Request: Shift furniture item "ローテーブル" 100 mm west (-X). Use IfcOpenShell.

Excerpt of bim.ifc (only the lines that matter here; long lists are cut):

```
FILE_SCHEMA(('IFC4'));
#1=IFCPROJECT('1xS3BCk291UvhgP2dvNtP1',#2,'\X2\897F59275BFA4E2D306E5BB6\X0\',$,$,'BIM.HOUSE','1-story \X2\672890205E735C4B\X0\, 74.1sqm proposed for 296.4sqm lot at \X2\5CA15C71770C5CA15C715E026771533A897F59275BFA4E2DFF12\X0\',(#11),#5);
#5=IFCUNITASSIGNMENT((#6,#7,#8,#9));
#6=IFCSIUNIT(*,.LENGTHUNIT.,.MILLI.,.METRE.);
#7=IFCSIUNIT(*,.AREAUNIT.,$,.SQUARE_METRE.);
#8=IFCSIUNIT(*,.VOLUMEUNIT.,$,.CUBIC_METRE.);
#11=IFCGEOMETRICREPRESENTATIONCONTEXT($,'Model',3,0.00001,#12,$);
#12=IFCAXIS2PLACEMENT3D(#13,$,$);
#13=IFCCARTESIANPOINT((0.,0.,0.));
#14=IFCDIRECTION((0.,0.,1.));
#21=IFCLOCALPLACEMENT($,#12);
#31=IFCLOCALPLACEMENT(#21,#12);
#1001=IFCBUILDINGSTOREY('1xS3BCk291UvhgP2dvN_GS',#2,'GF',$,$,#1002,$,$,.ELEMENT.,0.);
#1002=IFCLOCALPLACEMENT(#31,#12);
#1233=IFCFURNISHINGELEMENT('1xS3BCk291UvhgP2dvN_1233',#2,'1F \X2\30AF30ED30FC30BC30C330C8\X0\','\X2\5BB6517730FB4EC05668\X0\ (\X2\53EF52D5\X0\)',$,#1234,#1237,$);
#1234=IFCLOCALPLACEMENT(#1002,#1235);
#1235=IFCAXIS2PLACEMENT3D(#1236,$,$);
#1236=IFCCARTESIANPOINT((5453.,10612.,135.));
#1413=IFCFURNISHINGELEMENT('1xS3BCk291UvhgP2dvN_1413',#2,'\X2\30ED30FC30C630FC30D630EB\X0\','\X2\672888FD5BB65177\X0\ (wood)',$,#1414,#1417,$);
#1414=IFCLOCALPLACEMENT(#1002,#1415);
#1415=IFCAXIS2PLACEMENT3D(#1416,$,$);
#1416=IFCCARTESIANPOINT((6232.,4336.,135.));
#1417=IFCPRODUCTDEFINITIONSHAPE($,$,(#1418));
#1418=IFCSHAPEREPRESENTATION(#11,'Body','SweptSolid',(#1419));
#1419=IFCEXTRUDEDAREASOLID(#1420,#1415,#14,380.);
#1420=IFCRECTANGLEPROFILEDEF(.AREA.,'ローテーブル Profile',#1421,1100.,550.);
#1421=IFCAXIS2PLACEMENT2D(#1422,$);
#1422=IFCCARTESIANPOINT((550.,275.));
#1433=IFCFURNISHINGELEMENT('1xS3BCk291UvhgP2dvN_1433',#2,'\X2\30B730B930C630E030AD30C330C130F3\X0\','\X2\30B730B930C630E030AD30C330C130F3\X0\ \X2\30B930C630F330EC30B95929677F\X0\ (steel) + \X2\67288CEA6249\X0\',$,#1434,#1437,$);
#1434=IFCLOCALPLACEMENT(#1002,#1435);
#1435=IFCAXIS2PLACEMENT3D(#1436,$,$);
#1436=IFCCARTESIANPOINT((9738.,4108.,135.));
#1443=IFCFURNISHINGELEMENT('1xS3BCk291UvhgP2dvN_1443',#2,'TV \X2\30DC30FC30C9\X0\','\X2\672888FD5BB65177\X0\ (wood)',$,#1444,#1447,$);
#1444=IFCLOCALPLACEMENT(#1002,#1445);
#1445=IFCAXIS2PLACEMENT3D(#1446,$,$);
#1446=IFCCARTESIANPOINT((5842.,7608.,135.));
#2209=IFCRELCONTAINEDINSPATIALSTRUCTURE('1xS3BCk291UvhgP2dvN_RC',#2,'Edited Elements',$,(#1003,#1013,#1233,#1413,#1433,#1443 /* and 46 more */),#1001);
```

```python
import ifcopenshell
import ifcopenshell.api.geometry
import ifcopenshell.util.placement

model = ifcopenshell.open("bim.ifc")

item = model.by_guid("1xS3BCk291UvhgP2dvN_1413")
matrix = ifcopenshell.util.placement.get_local_placement(item.ObjectPlacement)
matrix[0, 3] -= 100.0
ifcopenshell.api.geometry.edit_object_placement(model, product=item, matrix=matrix, is_si=False)

print(ifcopenshell.util.placement.get_local_placement(item.ObjectPlacement).round(3) + 0.0)

model.write("bim_edited.ifc")
```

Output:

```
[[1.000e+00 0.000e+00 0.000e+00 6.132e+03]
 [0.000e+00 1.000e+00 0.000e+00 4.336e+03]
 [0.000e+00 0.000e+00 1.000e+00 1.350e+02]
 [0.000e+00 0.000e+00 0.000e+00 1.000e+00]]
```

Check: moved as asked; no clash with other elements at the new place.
